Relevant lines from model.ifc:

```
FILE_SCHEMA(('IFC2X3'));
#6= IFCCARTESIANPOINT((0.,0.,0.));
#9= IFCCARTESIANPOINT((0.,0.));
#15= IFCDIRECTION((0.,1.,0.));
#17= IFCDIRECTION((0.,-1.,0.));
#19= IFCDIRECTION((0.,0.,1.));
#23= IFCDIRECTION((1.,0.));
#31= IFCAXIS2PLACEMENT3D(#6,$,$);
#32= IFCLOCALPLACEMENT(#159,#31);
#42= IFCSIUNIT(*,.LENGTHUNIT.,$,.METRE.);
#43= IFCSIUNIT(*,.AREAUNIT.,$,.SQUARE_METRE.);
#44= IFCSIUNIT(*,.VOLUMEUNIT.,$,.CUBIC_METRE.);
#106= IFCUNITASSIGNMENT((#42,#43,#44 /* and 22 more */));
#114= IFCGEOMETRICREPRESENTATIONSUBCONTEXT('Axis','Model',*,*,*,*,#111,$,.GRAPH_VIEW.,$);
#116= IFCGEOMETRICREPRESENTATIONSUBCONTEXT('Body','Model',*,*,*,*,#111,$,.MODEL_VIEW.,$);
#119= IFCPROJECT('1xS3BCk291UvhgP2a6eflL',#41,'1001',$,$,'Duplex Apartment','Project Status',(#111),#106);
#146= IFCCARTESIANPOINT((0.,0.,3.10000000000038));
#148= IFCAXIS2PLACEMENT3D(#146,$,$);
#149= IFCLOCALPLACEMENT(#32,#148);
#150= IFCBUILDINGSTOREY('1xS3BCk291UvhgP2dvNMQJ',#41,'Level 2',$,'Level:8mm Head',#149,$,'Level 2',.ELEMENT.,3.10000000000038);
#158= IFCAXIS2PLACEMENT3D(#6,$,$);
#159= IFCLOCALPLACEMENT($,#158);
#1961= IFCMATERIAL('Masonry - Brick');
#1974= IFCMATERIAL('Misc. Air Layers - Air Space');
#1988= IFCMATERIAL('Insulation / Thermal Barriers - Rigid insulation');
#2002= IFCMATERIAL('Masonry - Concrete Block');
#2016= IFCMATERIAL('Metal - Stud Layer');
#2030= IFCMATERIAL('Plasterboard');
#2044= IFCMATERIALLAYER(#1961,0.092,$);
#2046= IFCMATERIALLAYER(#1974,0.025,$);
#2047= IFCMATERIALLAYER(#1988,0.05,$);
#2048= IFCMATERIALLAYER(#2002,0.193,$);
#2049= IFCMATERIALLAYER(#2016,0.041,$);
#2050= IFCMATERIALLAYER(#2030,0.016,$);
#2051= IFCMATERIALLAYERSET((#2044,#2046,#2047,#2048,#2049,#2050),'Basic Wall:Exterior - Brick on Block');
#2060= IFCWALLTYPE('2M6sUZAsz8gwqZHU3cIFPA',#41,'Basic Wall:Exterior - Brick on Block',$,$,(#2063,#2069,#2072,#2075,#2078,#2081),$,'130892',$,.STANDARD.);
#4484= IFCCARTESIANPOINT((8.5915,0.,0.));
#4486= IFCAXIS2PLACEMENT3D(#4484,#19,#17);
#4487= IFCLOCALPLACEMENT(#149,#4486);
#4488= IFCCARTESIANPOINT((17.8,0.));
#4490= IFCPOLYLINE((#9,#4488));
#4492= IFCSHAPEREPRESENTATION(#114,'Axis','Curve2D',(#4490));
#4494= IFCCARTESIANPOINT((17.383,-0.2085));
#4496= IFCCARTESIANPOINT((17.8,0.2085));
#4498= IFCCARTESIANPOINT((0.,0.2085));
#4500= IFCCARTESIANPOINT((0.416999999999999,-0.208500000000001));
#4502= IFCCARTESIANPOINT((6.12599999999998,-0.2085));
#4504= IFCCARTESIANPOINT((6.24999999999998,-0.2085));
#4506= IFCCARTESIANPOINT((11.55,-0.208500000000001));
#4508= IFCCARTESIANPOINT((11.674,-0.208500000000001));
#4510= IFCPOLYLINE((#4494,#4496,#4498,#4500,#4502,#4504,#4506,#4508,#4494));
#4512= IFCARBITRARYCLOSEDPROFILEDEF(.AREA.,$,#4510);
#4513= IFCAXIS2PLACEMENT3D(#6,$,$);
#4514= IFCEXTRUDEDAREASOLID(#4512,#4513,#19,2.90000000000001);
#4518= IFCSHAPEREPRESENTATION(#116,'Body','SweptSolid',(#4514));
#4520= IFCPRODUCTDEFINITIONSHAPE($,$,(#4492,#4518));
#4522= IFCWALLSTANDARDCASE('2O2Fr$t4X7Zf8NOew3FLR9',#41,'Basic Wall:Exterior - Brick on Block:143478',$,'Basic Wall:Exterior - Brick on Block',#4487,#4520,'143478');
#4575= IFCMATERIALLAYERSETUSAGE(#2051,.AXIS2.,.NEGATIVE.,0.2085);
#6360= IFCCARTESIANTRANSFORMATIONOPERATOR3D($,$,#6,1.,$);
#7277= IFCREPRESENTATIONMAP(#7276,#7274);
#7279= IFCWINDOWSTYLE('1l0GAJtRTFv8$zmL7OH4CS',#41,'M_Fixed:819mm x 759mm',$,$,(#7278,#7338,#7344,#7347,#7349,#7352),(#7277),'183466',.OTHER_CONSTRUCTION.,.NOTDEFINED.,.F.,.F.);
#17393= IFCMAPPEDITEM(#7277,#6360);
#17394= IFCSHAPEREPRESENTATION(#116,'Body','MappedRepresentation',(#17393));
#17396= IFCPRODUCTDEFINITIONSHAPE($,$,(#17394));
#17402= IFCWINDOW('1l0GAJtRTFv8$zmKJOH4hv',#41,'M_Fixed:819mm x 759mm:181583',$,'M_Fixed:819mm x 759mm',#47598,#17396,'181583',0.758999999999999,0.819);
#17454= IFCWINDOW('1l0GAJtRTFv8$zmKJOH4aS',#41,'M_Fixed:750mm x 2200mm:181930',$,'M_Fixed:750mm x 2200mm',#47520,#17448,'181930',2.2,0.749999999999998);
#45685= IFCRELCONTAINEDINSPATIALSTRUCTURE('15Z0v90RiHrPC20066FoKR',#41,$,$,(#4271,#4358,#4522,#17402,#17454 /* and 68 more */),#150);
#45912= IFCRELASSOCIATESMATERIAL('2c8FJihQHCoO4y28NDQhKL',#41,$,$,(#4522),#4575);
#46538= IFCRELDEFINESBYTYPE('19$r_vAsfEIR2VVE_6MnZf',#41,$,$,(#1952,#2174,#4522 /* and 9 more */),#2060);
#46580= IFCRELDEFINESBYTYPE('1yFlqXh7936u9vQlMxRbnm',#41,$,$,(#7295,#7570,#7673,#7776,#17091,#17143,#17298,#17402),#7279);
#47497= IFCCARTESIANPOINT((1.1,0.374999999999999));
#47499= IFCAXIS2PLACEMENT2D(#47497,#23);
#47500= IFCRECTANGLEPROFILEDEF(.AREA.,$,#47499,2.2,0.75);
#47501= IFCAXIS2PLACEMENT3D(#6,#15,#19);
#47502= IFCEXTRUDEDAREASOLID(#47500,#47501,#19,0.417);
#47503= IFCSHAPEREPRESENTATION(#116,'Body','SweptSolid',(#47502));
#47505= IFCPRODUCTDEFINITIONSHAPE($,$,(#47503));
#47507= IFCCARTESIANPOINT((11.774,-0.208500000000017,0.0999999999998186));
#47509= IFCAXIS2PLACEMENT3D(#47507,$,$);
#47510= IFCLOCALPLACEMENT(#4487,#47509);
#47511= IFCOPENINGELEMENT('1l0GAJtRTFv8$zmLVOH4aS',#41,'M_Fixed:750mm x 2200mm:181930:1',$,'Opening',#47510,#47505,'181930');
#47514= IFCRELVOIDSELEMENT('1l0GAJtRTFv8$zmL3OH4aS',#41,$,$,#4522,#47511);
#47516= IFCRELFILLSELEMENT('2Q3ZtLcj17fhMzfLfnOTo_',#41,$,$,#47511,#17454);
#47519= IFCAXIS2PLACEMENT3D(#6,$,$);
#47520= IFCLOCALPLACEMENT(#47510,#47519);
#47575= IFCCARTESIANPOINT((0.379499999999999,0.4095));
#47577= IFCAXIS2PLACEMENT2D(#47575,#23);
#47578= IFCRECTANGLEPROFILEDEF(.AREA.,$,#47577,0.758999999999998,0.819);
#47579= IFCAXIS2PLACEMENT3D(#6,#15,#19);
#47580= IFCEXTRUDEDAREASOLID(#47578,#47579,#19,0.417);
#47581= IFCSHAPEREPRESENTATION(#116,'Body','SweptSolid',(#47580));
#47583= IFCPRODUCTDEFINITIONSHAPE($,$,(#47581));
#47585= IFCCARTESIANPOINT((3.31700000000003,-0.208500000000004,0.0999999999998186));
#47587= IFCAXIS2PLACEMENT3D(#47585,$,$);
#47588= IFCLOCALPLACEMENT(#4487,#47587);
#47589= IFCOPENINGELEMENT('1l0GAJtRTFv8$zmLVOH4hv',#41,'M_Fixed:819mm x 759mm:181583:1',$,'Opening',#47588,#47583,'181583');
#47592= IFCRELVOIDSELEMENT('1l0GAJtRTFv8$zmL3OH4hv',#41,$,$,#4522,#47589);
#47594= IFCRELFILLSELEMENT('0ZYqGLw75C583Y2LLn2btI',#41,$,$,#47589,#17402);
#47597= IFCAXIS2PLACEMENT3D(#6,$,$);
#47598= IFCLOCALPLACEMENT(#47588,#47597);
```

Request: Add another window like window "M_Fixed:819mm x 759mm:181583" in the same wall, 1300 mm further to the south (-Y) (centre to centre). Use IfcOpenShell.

```python
import ifcopenshell
import ifcopenshell.api.feature
import ifcopenshell.api.geometry
import ifcopenshell.api.root
import ifcopenshell.geom
import ifcopenshell.util.element
import ifcopenshell.util.placement
import ifcopenshell.util.shape
import ifcopenshell.util.unit

model = ifcopenshell.open("model.ifc")
unit_scale = ifcopenshell.util.unit.calculate_unit_scale(model)
settings = ifcopenshell.geom.settings()


def volume(element):
    """Net volume in cubic metres, openings subtracted."""
    shape = ifcopenshell.geom.create_shape(settings, element)
    return ifcopenshell.util.shape.get_volume(shape.geometry)


def reuse_history(source, copy):
    """copy_class also copies each property set's owner history, people and application; keep the originals."""
    for rel in copy.IsDefinedBy:
        if rel.is_a("IfcRelDefinesByProperties") and (history := rel.RelatingPropertyDefinition.OwnerHistory):
            rel.RelatingPropertyDefinition.OwnerHistory = source.OwnerHistory
            ifcopenshell.util.element.remove_deep2(model, history)


window = model.by_guid("1l0GAJtRTFv8$zmKJOH4hv")
opening = window.FillsVoids[0].RelatingOpeningElement
wall = opening.VoidsElements[0].RelatingBuildingElement
before = volume(wall)
shift = ifcopenshell.util.placement.get_local_placement(wall.ObjectPlacement)[:3, 0] * 1.3 / unit_scale

# copy_class copies the void relationship, type, container and properties, but no geometry.
new_opening = ifcopenshell.api.root.copy_class(model, product=opening)
new_opening.Representation = ifcopenshell.util.element.copy_deep(
    model, opening.Representation, exclude=["IfcGeometricRepresentationContext", "IfcRepresentationMap"]
)
new_opening.Name = "M_Fixed:819mm x 759mm"
new_opening.Tag = None
new_window = ifcopenshell.api.root.copy_class(model, product=window)
new_window.Representation = ifcopenshell.util.element.copy_deep(
    model, window.Representation, exclude=["IfcGeometricRepresentationContext", "IfcRepresentationMap"]
)
new_window.Name = "M_Fixed:819mm x 759mm"
new_window.Tag = None
reuse_history(window, new_window)
fills = ifcopenshell.api.feature.add_filling(model, opening=new_opening, element=new_window)
fills.OwnerHistory = new_window.OwnerHistory  # required in IFC2X3

for old, new in ((opening, new_opening), (window, new_window)):
    matrix = ifcopenshell.util.placement.get_local_placement(old.ObjectPlacement)
    matrix[:3, 3] += shift
    ifcopenshell.api.geometry.edit_object_placement(model, product=new, matrix=matrix, is_si=False)

after = volume(wall)

print(f"wall volume {before:.3f} -> {after:.3f} m3")

model.write("model-out.ifc")
```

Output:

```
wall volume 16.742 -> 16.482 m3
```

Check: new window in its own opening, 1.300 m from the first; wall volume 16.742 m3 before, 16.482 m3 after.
